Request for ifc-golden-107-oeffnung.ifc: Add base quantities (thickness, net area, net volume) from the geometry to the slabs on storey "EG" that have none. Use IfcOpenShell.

First a look at what the model holds.

```python
import ifcopenshell
import ifcopenshell.util.element
import ifcopenshell.util.unit

model = ifcopenshell.open("ifc-golden-107-oeffnung.ifc")
print(model.schema)
for unit_type in ("LENGTHUNIT", "AREAUNIT", "VOLUMEUNIT"):
    print(unit_type, ifcopenshell.util.unit.calculate_unit_scale(model, unit_type))
storey = next(s for s in model.by_type("IfcBuildingStorey") if s.Name == "EG")
slabs = [e for e in ifcopenshell.util.element.get_decomposition(storey) if e.is_a("IfcSlab")]
for e in sorted(slabs, key=lambda e: e.id()):
    print(e.id(), e.is_a(), e.Name, list(ifcopenshell.util.element.get_psets(e, qtos_only=True)), sep=" | ")
```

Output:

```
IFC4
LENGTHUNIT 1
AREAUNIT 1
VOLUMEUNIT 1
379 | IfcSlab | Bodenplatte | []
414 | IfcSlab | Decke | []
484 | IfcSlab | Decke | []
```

```python
import ifcopenshell
import ifcopenshell.api.pset
import ifcopenshell.geom
import ifcopenshell.util.element
import ifcopenshell.util.shape
import ifcopenshell.util.unit

model = ifcopenshell.open("ifc-golden-107-oeffnung.ifc")
unit_scale = ifcopenshell.util.unit.calculate_unit_scale(model)
area_scale = ifcopenshell.util.unit.calculate_unit_scale(model, "AREAUNIT")
volume_scale = ifcopenshell.util.unit.calculate_unit_scale(model, "VOLUMEUNIT")
settings = ifcopenshell.geom.settings()

storey = next(s for s in model.by_type("IfcBuildingStorey") if s.Name == "EG")
slabs = [e for e in ifcopenshell.util.element.get_decomposition(storey) if e.is_a("IfcSlab")]

for e in sorted(slabs, key=lambda e: e.id()):
    if ifcopenshell.util.element.get_psets(e, qtos_only=True, should_inherit=False):
        continue
    # Geometry comes back in metres, in the element's own axes.
    shape = ifcopenshell.geom.create_shape(settings, e)
    values = {
        "Width": ifcopenshell.util.shape.get_z(shape.geometry) / unit_scale,
        "NetArea": ifcopenshell.util.shape.get_footprint_area(shape.geometry) / area_scale,
        "NetVolume": ifcopenshell.util.shape.get_volume(shape.geometry) / volume_scale,
    }
    qto = ifcopenshell.api.pset.add_qto(model, product=e, name="Qto_SlabBaseQuantities")
    ifcopenshell.api.pset.edit_qto(model, qto=qto, properties=values)
    print(e.id(), {k: round(v, 3) for k, v in values.items()})

model.write("ifc-golden-107-oeffnung_v2.ifc")
```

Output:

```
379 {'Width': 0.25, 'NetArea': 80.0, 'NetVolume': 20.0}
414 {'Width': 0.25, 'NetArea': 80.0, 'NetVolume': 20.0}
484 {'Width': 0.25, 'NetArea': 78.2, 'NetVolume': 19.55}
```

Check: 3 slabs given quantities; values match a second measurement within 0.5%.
